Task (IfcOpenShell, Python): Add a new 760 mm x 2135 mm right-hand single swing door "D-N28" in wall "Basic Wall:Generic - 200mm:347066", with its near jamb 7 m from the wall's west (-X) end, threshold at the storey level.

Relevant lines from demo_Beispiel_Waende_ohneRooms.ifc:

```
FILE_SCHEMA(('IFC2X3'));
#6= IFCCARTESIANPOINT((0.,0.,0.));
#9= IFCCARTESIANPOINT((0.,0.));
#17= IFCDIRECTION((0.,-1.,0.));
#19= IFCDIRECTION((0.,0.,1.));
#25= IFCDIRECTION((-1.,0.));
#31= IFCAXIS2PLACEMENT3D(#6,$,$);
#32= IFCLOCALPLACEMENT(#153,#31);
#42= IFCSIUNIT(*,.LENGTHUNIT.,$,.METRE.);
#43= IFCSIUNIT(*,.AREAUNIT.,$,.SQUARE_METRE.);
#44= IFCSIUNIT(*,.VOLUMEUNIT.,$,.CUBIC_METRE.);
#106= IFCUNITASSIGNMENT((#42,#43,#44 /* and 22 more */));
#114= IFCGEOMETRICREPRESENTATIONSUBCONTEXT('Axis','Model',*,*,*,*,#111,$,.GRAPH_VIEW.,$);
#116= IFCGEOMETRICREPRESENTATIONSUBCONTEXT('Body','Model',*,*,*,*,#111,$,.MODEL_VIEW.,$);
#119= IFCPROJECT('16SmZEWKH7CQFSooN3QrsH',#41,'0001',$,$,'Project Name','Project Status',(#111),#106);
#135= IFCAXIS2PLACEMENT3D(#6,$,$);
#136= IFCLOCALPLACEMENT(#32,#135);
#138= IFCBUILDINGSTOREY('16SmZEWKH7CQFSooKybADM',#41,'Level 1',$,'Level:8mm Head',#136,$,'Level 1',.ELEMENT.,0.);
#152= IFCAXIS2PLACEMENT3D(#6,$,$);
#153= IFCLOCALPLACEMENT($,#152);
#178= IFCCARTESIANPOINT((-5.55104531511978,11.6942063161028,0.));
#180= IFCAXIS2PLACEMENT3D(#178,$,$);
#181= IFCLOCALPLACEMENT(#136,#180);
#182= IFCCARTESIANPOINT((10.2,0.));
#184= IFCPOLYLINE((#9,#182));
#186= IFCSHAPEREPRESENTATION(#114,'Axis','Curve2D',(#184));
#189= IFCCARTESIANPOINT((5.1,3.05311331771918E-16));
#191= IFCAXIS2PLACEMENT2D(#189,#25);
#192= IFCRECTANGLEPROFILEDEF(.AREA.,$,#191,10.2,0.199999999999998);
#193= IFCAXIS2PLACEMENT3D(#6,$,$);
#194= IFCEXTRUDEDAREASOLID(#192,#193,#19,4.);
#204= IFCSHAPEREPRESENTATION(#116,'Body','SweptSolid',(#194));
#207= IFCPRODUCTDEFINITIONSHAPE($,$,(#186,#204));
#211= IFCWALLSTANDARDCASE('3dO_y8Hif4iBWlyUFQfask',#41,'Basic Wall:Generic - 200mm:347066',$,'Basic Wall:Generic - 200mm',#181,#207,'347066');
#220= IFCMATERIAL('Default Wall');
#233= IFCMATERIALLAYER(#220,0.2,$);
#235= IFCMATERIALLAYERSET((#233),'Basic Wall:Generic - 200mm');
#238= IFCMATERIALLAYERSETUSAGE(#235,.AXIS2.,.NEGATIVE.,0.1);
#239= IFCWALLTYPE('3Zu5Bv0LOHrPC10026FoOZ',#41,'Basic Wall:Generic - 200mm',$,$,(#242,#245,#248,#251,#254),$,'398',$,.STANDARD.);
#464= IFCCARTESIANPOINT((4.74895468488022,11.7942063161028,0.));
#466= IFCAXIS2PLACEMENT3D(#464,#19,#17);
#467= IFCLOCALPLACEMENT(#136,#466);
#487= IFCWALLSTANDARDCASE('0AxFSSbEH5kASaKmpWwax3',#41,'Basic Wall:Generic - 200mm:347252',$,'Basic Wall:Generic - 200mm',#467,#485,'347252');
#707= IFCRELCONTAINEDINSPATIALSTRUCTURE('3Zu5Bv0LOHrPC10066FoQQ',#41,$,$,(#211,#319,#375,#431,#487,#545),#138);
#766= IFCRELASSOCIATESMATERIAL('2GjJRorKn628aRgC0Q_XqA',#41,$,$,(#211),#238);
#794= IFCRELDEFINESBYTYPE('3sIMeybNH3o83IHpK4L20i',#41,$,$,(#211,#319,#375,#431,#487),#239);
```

```python
import numpy as np
import ifcopenshell
import ifcopenshell.api.feature
import ifcopenshell.api.geometry
import ifcopenshell.api.root
import ifcopenshell.api.spatial
import ifcopenshell.api.type
import ifcopenshell.geom
import ifcopenshell.util.element
import ifcopenshell.util.placement
import ifcopenshell.util.representation
import ifcopenshell.util.shape
import ifcopenshell.util.unit

model = ifcopenshell.open("demo_Beispiel_Waende_ohneRooms.ifc")
unit_scale = ifcopenshell.util.unit.calculate_unit_scale(model)
settings = ifcopenshell.geom.settings()


def volume(element):
    """Net volume in cubic metres, openings subtracted."""
    shape = ifcopenshell.geom.create_shape(settings, element)
    return ifcopenshell.util.shape.get_volume(shape.geometry)


wall = model.by_guid("3dO_y8Hif4iBWlyUFQfask")
storey = ifcopenshell.util.element.get_container(wall, ifc_class="IfcBuildingStorey")
context = ifcopenshell.util.representation.get_context(model, "Model", "Body", "MODEL_VIEW")
before = volume(wall)

width, height, from_end, sill = 0.76, 2.135, 7, 0.0  # metres

# The wall runs along its own X axis, and the end named is its -X end.
wall_shape = ifcopenshell.geom.create_shape(settings, wall)
x, y, z = ifcopenshell.util.shape.get_vertices(wall_shape.geometry).T
start = x.min() + from_end
face, thickness = float(y.min()), float(y.max() - y.min())
wall_matrix = ifcopenshell.util.placement.get_local_placement(wall.ObjectPlacement)
level = ifcopenshell.util.placement.get_local_placement(storey.ObjectPlacement)[2, 3]


def in_wall(x, y):
    """Placement at x, y metres in the wall's axes, at sill height."""
    matrix = wall_matrix.copy()
    matrix[:, 3] = wall_matrix @ np.array([x / unit_scale, y / unit_scale, 0.0, 1.0])
    matrix[2, 3] = level + sill / unit_scale
    return matrix


# Opening: a box that overshoots both wall faces by 50 mm.
opening = ifcopenshell.api.root.create_entity(model, ifc_class="IfcOpeningElement")
box = ifcopenshell.api.geometry.add_wall_representation(
    model, context=context, length=width, height=height, thickness=thickness + 0.1
)
ifcopenshell.api.geometry.assign_representation(model, product=opening, representation=box)
ifcopenshell.api.geometry.edit_object_placement(model, product=opening, matrix=in_wall(start, face - 0.05), is_si=False)
ifcopenshell.api.feature.add_feature(model, feature=opening, element=wall)

door = ifcopenshell.api.root.create_entity(model, ifc_class="IfcDoor", name="D-N28")
door.OverallWidth, door.OverallHeight = width / unit_scale, height / unit_scale
body = ifcopenshell.api.geometry.add_door_representation(
    model,
    context=context,
    overall_width=door.OverallWidth,
    overall_height=door.OverallHeight,
    operation_type="SINGLE_SWING_RIGHT",
    lining_properties={"LiningDepth": thickness / unit_scale, "ThresholdDepth": thickness / unit_scale},
)
ifcopenshell.api.geometry.assign_representation(model, product=door, representation=body)
ifcopenshell.api.spatial.assign_container(model, products=[door], relating_structure=storey)
fills = ifcopenshell.api.feature.add_filling(model, opening=opening, element=door)
fills.OwnerHistory = door.OwnerHistory  # required in IFC2X3

# IFC2X3 keeps the operation on the door style.
style = ifcopenshell.api.root.create_entity(model, ifc_class="IfcDoorStyle", name="D-N28")
style.OperationType, style.ConstructionType = "SINGLE_SWING_RIGHT", "NOTDEFINED"
style.ParameterTakesPrecedence = style.Sizeable = False
ifcopenshell.api.type.assign_type(model, related_objects=[door], relating_type=style)

# The lining spans the wall, so the door starts at the wall face.
ifcopenshell.api.geometry.edit_object_placement(model, product=door, matrix=in_wall(start, face), is_si=False)

after = volume(wall)

print(f"wall volume {before:.3f} -> {after:.3f} m3")

model.write("demo_Beispiel_Waende_ohneRooms_updated.ifc")
```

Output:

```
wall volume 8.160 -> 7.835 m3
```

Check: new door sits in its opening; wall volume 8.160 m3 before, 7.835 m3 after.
